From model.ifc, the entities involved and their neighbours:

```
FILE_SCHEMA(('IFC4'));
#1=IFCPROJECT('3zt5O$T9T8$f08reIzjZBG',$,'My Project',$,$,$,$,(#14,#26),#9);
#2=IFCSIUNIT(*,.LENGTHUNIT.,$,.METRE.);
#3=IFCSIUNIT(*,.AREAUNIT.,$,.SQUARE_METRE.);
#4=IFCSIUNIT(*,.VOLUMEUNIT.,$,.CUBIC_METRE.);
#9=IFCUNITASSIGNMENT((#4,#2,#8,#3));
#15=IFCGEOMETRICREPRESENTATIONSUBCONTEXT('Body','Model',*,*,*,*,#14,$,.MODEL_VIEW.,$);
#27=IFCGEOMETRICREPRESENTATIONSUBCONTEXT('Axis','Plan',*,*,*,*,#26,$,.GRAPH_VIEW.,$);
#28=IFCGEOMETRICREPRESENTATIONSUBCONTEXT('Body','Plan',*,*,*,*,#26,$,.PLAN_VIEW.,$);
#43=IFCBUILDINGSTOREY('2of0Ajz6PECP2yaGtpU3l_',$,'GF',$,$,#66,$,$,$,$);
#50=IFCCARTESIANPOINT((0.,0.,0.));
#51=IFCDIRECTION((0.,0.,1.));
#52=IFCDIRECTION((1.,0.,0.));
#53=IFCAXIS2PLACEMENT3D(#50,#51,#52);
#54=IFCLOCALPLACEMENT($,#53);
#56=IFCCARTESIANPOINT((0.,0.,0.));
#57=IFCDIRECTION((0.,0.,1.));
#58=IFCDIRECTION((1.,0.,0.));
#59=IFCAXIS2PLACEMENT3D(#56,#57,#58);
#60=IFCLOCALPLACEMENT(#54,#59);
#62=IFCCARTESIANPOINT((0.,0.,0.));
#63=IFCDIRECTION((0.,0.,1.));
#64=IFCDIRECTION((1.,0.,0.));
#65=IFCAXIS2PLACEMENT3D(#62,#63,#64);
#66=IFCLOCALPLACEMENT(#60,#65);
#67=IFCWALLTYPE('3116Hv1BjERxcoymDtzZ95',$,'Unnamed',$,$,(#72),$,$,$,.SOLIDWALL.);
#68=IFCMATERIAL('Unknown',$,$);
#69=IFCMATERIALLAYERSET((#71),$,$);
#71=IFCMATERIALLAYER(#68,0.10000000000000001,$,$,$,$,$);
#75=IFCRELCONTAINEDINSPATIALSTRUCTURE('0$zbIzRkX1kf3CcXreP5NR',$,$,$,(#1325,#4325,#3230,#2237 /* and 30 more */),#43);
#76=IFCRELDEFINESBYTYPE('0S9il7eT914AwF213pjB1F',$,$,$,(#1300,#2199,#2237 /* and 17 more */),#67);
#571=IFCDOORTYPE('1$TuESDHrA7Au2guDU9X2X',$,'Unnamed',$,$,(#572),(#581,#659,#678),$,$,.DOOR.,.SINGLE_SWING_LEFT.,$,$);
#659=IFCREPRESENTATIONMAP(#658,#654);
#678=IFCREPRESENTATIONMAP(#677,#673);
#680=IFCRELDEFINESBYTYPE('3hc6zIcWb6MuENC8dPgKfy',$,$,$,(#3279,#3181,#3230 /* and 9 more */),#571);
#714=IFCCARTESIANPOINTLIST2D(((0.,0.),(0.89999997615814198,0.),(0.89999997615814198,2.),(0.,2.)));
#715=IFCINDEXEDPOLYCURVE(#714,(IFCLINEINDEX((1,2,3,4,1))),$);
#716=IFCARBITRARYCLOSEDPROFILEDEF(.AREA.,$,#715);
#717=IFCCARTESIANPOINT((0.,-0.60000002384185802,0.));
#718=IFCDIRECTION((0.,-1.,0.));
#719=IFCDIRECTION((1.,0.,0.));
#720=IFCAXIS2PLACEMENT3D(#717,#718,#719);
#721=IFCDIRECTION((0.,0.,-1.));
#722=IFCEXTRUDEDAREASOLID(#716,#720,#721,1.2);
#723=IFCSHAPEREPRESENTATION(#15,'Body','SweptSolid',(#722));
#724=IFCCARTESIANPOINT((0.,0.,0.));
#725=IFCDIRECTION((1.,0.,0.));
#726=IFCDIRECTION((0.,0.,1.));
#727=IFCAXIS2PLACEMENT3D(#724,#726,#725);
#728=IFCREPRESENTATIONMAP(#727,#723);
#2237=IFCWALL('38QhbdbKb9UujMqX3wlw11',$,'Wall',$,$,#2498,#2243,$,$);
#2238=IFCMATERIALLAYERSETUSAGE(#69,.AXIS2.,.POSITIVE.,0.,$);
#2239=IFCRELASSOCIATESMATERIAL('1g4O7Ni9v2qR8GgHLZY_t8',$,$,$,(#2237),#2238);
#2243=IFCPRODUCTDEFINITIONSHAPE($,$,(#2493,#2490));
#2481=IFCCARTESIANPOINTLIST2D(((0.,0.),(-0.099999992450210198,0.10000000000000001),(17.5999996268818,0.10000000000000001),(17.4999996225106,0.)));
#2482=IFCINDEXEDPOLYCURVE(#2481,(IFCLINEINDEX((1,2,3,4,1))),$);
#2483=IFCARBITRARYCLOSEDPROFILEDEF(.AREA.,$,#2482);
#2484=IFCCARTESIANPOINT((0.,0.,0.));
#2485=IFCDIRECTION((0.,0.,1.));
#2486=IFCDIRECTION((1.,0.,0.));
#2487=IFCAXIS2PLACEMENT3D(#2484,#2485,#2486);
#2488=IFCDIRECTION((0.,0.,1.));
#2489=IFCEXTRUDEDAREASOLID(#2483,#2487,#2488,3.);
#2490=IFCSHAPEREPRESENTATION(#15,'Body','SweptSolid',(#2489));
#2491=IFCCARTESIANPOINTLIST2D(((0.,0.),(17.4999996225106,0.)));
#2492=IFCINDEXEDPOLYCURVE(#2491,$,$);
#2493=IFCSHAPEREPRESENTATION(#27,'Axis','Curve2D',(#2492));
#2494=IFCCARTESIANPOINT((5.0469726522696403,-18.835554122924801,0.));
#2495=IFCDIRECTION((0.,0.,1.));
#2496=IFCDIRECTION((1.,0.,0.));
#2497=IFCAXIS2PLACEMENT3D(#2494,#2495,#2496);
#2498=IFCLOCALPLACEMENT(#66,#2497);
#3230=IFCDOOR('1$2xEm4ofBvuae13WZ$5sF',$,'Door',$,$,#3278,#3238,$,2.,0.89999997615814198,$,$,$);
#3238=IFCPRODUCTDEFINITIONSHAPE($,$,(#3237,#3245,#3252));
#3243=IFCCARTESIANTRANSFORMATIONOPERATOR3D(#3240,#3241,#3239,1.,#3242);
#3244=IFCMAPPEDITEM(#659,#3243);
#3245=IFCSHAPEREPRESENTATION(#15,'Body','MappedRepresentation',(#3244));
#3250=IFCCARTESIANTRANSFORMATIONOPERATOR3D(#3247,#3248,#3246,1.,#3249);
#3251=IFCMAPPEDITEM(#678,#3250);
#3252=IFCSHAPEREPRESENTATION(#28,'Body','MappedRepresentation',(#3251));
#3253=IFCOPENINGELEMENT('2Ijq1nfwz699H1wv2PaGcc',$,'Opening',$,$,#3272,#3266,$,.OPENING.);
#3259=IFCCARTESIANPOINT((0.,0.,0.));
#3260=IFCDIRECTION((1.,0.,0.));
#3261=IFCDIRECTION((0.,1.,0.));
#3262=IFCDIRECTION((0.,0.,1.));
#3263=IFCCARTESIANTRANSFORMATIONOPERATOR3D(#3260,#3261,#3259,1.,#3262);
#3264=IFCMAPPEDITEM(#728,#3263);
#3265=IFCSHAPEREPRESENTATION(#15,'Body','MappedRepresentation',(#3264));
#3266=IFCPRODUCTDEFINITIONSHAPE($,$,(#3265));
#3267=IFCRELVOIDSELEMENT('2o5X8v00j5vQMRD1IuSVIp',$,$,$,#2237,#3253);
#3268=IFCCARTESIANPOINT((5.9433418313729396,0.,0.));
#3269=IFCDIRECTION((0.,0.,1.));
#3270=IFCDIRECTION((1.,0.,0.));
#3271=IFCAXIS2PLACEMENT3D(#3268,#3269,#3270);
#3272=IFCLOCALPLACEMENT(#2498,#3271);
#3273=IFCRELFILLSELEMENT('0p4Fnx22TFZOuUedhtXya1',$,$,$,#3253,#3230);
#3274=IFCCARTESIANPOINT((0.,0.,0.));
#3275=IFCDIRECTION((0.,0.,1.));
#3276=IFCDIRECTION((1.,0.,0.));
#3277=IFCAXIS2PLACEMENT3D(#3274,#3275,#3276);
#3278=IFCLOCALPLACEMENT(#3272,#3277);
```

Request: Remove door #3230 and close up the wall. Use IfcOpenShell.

```python
import ifcopenshell
import ifcopenshell.api.feature
import ifcopenshell.api.root
import ifcopenshell.geom
import ifcopenshell.util.shape

model = ifcopenshell.open("model.ifc")
settings = ifcopenshell.geom.settings()


def volume(element):
    """Net volume in cubic metres, openings subtracted."""
    shape = ifcopenshell.geom.create_shape(settings, element)
    return ifcopenshell.util.shape.get_volume(shape.geometry)


door = model.by_guid("1$2xEm4ofBvuae13WZ$5sF")
opening = door.FillsVoids[0].RelatingOpeningElement
wall = opening.VoidsElements[0].RelatingBuildingElement
before = volume(wall)

ifcopenshell.api.root.remove_product(model, product=door)
ifcopenshell.api.feature.remove_feature(model, feature=opening)

after = volume(wall)

print(f"wall volume {before:.3f} -> {after:.3f} m3")

model.write("model_v2.ifc")
```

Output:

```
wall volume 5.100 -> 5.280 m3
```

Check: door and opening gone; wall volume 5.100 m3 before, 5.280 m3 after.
